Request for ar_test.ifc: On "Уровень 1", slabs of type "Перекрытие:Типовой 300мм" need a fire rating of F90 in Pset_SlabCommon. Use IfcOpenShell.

First a look at what the model holds.

```python
import ifcopenshell
import ifcopenshell.util.element

model = ifcopenshell.open("ar_test.ifc")
print(model.schema)
storey = next(s for s in model.by_type("IfcBuildingStorey") if s.Name == "Уровень 1")
slabs = [e for e in ifcopenshell.util.element.get_decomposition(storey) if e.is_a("IfcSlab")]
seen = {}
for e in slabs:
    element_type = ifcopenshell.util.element.get_type(e)
    key = (element_type.Name if element_type != e and element_type else None, ifcopenshell.util.element.get_pset(e, "Pset_SlabCommon", "FireRating"))
    seen[key] = seen.get(key, 0) + 1
for (name, value), count in sorted(seen.items(), key=str):
    print(count, "x", name, "|", value)
```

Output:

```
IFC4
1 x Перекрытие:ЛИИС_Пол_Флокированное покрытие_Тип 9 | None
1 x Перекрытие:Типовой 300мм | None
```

```python
import ifcopenshell
import ifcopenshell.api.pset
import ifcopenshell.util.element

model = ifcopenshell.open("ar_test.ifc")

storey = next(s for s in model.by_type("IfcBuildingStorey") if s.Name == "Уровень 1")
slabs = [e for e in ifcopenshell.util.element.get_decomposition(storey) if e.is_a("IfcSlab")]

count = 0
for e in slabs:
    element_type = ifcopenshell.util.element.get_type(e)
    if element_type in (None, e) or element_type.Name != "Перекрытие:Типовой 300мм":
        continue
    # add_pset returns the element's existing set when there is one.
    pset = ifcopenshell.api.pset.add_pset(model, product=e, name="Pset_SlabCommon")
    ifcopenshell.api.pset.edit_pset(model, pset=pset, properties={"FireRating": "F90"})
    count += 1

print(count, "slabs updated")

model.write("ar_test_edited.ifc")
```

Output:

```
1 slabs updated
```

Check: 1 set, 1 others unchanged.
